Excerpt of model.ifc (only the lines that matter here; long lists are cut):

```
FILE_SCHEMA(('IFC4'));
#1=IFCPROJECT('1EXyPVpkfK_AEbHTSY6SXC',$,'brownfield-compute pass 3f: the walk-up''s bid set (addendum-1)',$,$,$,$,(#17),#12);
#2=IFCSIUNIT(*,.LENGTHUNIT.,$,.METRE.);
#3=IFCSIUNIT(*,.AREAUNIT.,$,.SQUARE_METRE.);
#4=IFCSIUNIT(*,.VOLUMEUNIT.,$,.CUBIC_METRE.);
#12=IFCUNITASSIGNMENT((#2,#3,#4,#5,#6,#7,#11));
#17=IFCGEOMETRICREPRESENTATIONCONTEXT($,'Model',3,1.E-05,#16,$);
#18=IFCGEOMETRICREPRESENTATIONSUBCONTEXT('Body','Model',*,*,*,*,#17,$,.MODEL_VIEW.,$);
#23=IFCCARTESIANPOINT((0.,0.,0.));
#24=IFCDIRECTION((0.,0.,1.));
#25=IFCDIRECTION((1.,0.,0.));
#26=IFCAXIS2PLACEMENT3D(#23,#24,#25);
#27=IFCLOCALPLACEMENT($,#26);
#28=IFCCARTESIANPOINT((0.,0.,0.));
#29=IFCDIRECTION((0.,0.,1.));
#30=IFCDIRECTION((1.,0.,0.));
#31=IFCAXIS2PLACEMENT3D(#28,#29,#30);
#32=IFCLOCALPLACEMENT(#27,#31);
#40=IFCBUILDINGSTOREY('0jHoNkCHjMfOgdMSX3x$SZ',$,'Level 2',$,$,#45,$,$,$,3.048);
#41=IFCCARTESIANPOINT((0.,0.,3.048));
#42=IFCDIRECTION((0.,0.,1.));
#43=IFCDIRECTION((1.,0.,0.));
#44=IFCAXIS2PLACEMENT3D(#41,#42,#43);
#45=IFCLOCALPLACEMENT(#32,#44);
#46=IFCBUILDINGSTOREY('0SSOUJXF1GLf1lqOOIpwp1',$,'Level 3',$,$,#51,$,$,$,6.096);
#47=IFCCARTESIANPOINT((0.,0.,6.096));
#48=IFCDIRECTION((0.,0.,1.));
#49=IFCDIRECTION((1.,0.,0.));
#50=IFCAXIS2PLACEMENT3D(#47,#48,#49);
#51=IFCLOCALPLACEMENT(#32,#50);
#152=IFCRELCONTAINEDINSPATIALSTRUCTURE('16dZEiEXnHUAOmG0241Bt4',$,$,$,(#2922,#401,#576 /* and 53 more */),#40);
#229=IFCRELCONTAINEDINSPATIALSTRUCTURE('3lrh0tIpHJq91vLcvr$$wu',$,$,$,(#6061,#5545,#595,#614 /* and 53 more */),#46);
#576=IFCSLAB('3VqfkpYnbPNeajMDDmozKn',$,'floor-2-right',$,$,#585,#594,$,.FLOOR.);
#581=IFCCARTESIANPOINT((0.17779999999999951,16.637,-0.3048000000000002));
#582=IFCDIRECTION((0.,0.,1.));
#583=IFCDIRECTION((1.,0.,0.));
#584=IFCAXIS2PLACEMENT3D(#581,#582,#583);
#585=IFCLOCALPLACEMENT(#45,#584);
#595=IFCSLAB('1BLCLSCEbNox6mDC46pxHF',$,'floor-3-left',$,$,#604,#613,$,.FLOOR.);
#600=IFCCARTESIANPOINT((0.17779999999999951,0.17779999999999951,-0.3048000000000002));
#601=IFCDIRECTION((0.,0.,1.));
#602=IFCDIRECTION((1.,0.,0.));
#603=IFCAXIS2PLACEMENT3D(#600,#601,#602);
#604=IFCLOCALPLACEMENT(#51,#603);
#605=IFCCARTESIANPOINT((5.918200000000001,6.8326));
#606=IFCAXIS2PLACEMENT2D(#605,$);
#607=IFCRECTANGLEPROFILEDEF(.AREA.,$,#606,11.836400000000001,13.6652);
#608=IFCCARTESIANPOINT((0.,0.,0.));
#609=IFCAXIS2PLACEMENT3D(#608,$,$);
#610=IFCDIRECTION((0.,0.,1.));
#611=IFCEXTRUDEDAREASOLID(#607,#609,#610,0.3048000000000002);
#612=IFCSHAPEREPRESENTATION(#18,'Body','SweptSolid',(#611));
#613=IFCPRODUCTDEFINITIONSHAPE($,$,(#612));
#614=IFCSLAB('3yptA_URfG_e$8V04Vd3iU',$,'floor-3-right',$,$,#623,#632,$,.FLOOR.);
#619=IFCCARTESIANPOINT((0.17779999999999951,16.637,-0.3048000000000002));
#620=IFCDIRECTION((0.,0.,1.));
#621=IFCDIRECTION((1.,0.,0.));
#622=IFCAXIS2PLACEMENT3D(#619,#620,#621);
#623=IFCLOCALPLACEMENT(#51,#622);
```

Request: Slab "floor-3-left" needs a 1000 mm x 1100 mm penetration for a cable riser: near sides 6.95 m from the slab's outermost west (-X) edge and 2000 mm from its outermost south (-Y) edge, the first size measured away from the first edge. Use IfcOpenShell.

```python
import numpy as np
import ifcopenshell
import ifcopenshell.api.feature
import ifcopenshell.api.geometry
import ifcopenshell.api.root
import ifcopenshell.geom
import ifcopenshell.util.placement
import ifcopenshell.util.representation
import ifcopenshell.util.shape
import ifcopenshell.util.unit

model = ifcopenshell.open("model.ifc")
unit_scale = ifcopenshell.util.unit.calculate_unit_scale(model)
settings = ifcopenshell.geom.settings()


def volume(element):
    """Net volume in cubic metres, openings subtracted."""
    shape = ifcopenshell.geom.create_shape(settings, element)
    return ifcopenshell.util.shape.get_volume(shape.geometry)


slab = model.by_guid("1BLCLSCEbNox6mDC46pxHF")
before = volume(slab)

# Extent in the slab's own axes, in metres. The edges named are its -X and -Y sides.
slab_shape = ifcopenshell.geom.create_shape(settings, slab)
vertices = ifcopenshell.util.shape.get_vertices(slab_shape.geometry)
x_min, y_min, bottom = vertices.min(axis=0)
top = vertices[:, 2].max()

opening = ifcopenshell.api.root.create_entity(model, ifc_class="IfcOpeningElement", name="Cable riser opening", predefined_type="OPENING")
context = ifcopenshell.util.representation.get_context(model, "Model", "Body", "MODEL_VIEW")
width, depth = 1, 1.1
outline = [(0.0, 0.0), (width, 0.0), (width, depth), (0.0, depth), (0.0, 0.0)]
# Overshoot both faces by 50 mm so the cut is clean.
shape = ifcopenshell.api.geometry.add_slab_representation(
    model, context=context, depth=top - bottom + 0.1, polyline=outline
)
ifcopenshell.api.geometry.assign_representation(model, product=opening, representation=shape)

matrix = ifcopenshell.util.placement.get_local_placement(slab.ObjectPlacement)
matrix[:, 3] = matrix @ np.append(np.array([x_min + 6.95, y_min + 2, bottom - 0.05]) / unit_scale, 1.0)
ifcopenshell.api.geometry.edit_object_placement(model, product=opening, matrix=matrix, is_si=False)
ifcopenshell.api.feature.add_feature(model, feature=opening, element=slab)

after = volume(slab)

print(f"slab volume {before:.3f} -> {after:.3f} m3")

model.write("model_edited.ifc")
```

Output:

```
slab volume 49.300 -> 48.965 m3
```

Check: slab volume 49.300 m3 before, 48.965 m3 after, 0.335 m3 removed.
